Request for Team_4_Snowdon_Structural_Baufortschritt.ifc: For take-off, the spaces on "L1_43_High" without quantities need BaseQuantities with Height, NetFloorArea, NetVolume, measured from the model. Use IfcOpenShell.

First a look at what the model holds.

```python
import ifcopenshell
import ifcopenshell.util.element
import ifcopenshell.util.unit

model = ifcopenshell.open("Team_4_Snowdon_Structural_Baufortschritt.ifc")
print(model.schema)
for unit_type in ("LENGTHUNIT", "AREAUNIT", "VOLUMEUNIT"):
    print(unit_type, ifcopenshell.util.unit.calculate_unit_scale(model, unit_type))
storey = next(s for s in model.by_type("IfcBuildingStorey") if s.Name == "L1_43_High")
spaces = [e for e in ifcopenshell.util.element.get_decomposition(storey) if e.is_a("IfcSpace")]
for e in sorted(spaces, key=lambda e: e.id()):
    print(e.id(), e.is_a(), e.Name, list(ifcopenshell.util.element.get_psets(e, qtos_only=True)), sep=" | ")
```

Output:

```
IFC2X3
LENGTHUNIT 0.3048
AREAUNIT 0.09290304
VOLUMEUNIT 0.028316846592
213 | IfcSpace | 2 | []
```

```python
import ifcopenshell
import ifcopenshell.api.pset
import ifcopenshell.geom
import ifcopenshell.util.element
import ifcopenshell.util.shape
import ifcopenshell.util.unit

model = ifcopenshell.open("Team_4_Snowdon_Structural_Baufortschritt.ifc")
unit_scale = ifcopenshell.util.unit.calculate_unit_scale(model)
area_scale = ifcopenshell.util.unit.calculate_unit_scale(model, "AREAUNIT")
volume_scale = ifcopenshell.util.unit.calculate_unit_scale(model, "VOLUMEUNIT")
settings = ifcopenshell.geom.settings()

storey = next(s for s in model.by_type("IfcBuildingStorey") if s.Name == "L1_43_High")
spaces = [e for e in ifcopenshell.util.element.get_decomposition(storey) if e.is_a("IfcSpace")]

for e in sorted(spaces, key=lambda e: e.id()):
    if ifcopenshell.util.element.get_psets(e, qtos_only=True, should_inherit=False):
        continue
    # Geometry comes back in metres, in the element's own axes.
    shape = ifcopenshell.geom.create_shape(settings, e)
    values = {
        "Height": ifcopenshell.util.shape.get_z(shape.geometry) / unit_scale,
        "NetFloorArea": ifcopenshell.util.shape.get_footprint_area(shape.geometry) / area_scale,
        "NetVolume": ifcopenshell.util.shape.get_volume(shape.geometry) / volume_scale,
    }
    qto = ifcopenshell.api.pset.add_qto(model, product=e, name="BaseQuantities")
    ifcopenshell.api.pset.edit_qto(model, qto=qto, properties=values)
    print(e.id(), {k: round(v, 3) for k, v in values.items()})

model.write("Team_4_Snowdon_Structural_Baufortschritt_edited.ifc")
```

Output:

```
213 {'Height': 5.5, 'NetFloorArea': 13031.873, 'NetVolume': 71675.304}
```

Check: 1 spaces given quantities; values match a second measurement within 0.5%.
